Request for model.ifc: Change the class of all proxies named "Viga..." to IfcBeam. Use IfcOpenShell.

First a look at what the model holds.

```python
import re

import ifcopenshell

model = ifcopenshell.open("model.ifc")
print(model.schema)
seen = {}
for e in model.by_type("IfcBuildingElementProxy"):
    name = re.sub(r":\d+(:\d+)?$", "", e.Name or "")  # drop the element id that some exporters append
    seen[name] = seen.get(name, 0) + 1
for name, count in sorted(seen.items()):
    print(count, "x", name)
```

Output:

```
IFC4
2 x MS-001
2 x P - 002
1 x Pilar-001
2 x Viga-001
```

```python
import ifcopenshell
import ifcopenshell.api.root

model = ifcopenshell.open("model.ifc")

proxies = [e.id() for e in model.by_type("IfcBuildingElementProxy") if (e.Name or "").startswith("Viga")]
for step_id in proxies:
    proxy = model.by_id(step_id)
    # Reclassifying a typed element also reclassifies its type and the type's other occurrences.
    if proxy.is_a("IfcBuildingElementProxy"):
        ifcopenshell.api.root.reassign_class(model, product=proxy, ifc_class="IfcBeam")

print(sum(model.by_id(i).is_a("IfcBeam") for i in proxies), "reclassified")

model.write("model_updated.ifc")
```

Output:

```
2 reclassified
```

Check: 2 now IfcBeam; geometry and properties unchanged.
